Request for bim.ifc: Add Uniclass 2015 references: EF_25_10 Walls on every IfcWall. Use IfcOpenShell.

First a look at what the model holds.

```python
import ifcopenshell

model = ifcopenshell.open("bim.ifc")
print(model.schema)
print("classifications:", [c.Name for c in model.by_type("IfcClassification")])
for ifc_class in ("IfcDoor", "IfcRoof", "IfcStair", "IfcWall", "IfcWindow"):
    print(ifc_class, len(model.by_type(ifc_class)))
```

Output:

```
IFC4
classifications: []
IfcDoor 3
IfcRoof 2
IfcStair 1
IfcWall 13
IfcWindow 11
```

```python
import ifcopenshell
import ifcopenshell.api.classification

model = ifcopenshell.open("bim.ifc")

system = ifcopenshell.api.classification.add_classification(model, classification="Uniclass 2015")

codes = {
    "IfcWall": ("EF_25_10", "Walls"),
}
for ifc_class, (code, name) in codes.items():
    products = model.by_type(ifc_class)
    ifcopenshell.api.classification.add_reference(
        model, products=products, classification=system, identification=code, name=name
    )
    print(code, len(products))

model.write("bim_v2.ifc")
```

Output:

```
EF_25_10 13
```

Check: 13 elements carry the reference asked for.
